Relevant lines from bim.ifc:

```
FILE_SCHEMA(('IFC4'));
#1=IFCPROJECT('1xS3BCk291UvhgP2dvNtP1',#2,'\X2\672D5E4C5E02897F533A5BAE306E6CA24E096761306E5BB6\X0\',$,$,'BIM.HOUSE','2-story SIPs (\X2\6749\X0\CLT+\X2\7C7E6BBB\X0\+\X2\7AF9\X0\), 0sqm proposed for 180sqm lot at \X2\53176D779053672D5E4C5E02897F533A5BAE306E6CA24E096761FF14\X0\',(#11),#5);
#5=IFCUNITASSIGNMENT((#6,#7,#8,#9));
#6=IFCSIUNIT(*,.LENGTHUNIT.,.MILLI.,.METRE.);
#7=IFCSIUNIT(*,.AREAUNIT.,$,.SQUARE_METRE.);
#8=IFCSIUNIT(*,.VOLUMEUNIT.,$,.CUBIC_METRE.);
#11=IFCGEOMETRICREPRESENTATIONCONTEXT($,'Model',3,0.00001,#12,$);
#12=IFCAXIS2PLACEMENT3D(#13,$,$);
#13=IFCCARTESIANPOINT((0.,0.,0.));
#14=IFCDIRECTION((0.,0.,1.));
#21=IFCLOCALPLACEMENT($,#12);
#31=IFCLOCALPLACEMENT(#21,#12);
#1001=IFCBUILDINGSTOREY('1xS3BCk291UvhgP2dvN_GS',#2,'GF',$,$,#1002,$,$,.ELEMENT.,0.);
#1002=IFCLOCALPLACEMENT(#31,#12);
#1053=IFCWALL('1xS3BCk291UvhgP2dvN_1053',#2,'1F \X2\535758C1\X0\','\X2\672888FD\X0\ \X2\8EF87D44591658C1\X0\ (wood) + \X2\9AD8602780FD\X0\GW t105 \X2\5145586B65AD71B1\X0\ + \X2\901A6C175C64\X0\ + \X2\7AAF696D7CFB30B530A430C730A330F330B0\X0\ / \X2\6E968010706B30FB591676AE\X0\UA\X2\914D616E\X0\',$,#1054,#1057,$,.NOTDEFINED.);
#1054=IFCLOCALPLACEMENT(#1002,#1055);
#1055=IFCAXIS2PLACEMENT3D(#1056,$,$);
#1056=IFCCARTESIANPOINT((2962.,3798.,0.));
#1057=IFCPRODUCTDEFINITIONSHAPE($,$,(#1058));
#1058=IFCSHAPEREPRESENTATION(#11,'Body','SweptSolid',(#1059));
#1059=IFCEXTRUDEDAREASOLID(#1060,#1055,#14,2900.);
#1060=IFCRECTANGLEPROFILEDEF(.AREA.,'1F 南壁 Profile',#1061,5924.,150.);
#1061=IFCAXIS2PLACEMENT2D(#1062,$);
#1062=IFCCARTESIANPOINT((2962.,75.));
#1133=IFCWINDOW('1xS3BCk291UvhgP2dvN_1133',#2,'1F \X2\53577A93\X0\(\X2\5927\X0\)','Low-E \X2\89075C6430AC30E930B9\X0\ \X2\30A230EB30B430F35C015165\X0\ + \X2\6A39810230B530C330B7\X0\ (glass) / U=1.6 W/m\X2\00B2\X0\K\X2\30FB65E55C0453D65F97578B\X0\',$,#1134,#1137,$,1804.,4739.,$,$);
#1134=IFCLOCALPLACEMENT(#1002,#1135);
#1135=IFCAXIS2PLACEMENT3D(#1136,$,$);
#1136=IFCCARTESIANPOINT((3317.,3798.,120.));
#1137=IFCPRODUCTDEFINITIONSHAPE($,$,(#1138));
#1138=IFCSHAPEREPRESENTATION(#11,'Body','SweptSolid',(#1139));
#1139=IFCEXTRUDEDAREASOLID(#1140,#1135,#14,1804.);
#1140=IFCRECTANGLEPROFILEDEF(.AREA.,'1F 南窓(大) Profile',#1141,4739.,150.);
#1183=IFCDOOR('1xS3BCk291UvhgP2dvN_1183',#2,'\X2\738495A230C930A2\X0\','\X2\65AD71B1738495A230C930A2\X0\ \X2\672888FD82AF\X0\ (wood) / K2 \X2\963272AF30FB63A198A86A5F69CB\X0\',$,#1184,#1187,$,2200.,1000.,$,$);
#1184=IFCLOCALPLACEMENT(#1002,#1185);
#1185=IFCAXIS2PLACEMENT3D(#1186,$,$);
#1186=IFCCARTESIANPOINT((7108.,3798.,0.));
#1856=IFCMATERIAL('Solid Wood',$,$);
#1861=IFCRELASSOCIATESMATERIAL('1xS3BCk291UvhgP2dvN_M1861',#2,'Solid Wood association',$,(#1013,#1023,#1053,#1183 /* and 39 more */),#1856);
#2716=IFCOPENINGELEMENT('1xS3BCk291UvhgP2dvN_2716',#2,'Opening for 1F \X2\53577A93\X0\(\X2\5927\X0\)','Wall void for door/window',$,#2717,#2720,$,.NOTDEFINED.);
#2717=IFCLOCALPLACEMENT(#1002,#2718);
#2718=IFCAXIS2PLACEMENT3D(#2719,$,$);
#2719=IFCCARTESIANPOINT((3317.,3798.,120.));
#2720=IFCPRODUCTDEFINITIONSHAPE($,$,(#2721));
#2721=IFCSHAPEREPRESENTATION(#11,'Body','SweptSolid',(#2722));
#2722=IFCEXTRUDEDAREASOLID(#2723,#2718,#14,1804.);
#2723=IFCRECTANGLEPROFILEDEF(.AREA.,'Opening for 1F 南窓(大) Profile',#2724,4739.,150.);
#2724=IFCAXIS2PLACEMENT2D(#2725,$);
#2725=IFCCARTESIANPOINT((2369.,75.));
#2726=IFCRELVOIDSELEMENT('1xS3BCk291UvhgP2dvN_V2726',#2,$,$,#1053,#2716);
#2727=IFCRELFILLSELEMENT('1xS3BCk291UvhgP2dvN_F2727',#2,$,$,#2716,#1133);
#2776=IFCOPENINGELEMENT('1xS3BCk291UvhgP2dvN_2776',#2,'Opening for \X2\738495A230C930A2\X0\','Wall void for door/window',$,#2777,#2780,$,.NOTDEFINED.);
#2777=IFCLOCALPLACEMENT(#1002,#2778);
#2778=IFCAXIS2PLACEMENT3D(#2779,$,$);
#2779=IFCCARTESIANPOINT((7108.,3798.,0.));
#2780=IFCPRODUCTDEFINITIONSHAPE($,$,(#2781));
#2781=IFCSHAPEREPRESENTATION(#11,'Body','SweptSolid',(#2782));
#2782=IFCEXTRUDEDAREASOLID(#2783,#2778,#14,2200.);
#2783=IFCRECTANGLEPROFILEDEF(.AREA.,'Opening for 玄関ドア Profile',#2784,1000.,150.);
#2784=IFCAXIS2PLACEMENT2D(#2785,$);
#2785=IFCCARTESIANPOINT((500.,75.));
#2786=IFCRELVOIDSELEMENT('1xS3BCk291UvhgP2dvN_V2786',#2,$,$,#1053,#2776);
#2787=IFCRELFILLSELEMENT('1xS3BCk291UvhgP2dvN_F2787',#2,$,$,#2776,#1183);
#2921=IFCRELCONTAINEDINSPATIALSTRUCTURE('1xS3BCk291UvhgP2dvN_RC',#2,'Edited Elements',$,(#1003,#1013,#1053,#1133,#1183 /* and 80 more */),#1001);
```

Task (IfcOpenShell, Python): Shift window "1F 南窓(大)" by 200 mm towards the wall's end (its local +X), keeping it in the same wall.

```python
import ifcopenshell
import ifcopenshell.api.geometry
import ifcopenshell.util.placement

model = ifcopenshell.open("bim.ifc")

window = model.by_guid("1xS3BCk291UvhgP2dvN_1133")
opening = window.FillsVoids[0].RelatingOpeningElement
wall = opening.VoidsElements[0].RelatingBuildingElement

wall_matrix = ifcopenshell.util.placement.get_local_placement(wall.ObjectPlacement)
shift = wall_matrix[:3, 0] * 200.0
before = ifcopenshell.util.placement.get_local_placement(window.ObjectPlacement)[:3, 3].copy()

# The window is not placed relative to its opening, so move both.
for product in (opening, window):
    matrix = ifcopenshell.util.placement.get_local_placement(product.ObjectPlacement)
    matrix[:3, 3] += shift
    ifcopenshell.api.geometry.edit_object_placement(model, product=product, matrix=matrix, is_si=False)

after = ifcopenshell.util.placement.get_local_placement(window.ObjectPlacement)[:3, 3]
print("window moved by", (after - before).round(3) + 0.0)

model.write("bim-out.ifc")
```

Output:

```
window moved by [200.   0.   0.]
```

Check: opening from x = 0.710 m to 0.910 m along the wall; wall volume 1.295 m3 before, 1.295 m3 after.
